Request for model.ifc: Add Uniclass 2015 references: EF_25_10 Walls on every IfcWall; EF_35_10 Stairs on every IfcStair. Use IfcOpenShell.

First a look at what the model holds.

```python
import ifcopenshell

model = ifcopenshell.open("model.ifc")
print(model.schema)
print("classifications:", [c.Name for c in model.by_type("IfcClassification")])
for ifc_class in ("IfcDoor", "IfcRoof", "IfcStair", "IfcWall", "IfcWindow"):
    print(ifc_class, len(model.by_type(ifc_class)))
```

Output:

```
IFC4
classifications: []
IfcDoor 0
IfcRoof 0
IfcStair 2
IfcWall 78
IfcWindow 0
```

```python
import ifcopenshell
import ifcopenshell.api.classification

model = ifcopenshell.open("model.ifc")

system = ifcopenshell.api.classification.add_classification(model, classification="Uniclass 2015")

codes = {
    "IfcWall": ("EF_25_10", "Walls"),
    "IfcStair": ("EF_35_10", "Stairs"),
}
for ifc_class, (code, name) in codes.items():
    products = model.by_type(ifc_class)
    ifcopenshell.api.classification.add_reference(
        model, products=products, classification=system, identification=code, name=name
    )
    print(code, len(products))

model.write("model_updated.ifc")
```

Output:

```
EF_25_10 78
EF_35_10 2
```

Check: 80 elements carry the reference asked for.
